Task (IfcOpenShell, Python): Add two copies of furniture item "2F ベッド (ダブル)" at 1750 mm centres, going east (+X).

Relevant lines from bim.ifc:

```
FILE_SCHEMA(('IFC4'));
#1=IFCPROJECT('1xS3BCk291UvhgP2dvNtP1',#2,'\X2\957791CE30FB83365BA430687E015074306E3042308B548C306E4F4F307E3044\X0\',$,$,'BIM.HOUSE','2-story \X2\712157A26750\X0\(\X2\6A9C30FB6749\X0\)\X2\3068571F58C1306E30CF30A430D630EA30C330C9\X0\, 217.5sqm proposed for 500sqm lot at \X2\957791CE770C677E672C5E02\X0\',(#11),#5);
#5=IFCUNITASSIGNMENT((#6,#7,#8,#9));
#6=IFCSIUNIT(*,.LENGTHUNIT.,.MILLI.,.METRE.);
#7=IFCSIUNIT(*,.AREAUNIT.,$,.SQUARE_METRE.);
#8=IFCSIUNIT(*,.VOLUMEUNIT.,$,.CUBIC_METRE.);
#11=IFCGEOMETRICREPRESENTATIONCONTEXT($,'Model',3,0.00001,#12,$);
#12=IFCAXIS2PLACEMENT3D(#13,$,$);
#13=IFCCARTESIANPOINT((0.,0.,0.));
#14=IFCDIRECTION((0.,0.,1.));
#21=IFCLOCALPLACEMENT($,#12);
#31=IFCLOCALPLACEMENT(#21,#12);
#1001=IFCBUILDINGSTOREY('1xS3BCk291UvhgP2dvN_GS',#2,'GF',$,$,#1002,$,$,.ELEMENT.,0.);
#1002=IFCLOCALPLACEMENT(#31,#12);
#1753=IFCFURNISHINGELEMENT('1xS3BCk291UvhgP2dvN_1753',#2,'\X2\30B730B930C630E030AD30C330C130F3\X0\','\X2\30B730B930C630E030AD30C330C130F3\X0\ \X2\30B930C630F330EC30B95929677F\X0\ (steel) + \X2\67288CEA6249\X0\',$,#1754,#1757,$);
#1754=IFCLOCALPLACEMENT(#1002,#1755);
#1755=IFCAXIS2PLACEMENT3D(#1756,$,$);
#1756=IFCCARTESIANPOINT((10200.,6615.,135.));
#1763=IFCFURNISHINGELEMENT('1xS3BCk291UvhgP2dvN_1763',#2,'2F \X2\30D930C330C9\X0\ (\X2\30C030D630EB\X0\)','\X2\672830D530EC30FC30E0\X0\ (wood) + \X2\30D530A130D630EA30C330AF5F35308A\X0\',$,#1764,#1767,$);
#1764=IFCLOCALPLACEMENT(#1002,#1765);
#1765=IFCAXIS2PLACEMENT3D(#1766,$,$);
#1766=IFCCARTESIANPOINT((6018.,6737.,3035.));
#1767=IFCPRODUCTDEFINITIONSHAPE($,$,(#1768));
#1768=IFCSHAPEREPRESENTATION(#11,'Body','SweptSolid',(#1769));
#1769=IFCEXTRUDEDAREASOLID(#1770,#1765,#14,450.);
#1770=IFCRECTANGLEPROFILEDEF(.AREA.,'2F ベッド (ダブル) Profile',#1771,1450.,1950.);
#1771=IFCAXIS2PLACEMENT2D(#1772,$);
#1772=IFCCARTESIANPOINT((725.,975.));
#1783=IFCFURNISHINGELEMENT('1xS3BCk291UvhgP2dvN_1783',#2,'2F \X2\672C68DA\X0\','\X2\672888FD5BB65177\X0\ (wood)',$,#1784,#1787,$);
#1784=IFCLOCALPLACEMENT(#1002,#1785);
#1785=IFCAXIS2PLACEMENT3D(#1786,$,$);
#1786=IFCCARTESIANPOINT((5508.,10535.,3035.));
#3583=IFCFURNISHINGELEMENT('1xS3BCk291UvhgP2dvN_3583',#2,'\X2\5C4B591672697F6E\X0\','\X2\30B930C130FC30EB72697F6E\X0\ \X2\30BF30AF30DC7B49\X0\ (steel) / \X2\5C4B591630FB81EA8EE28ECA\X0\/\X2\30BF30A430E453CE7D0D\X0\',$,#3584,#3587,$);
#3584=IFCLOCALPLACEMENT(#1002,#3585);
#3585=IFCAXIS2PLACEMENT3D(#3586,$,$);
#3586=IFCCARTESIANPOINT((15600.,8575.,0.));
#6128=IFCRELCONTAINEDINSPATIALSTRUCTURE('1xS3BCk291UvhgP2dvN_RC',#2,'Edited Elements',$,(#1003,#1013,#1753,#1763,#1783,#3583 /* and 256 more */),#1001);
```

```python
import numpy as np
import ifcopenshell
import ifcopenshell.api.geometry
import ifcopenshell.api.root
import ifcopenshell.util.element
import ifcopenshell.util.placement
import ifcopenshell.util.unit

model = ifcopenshell.open("bim.ifc")
unit_scale = ifcopenshell.util.unit.calculate_unit_scale(model)


def reuse_history(source, copy):
    """copy_class also copies each property set's owner history, people and application; keep the originals."""
    for rel in copy.IsDefinedBy:
        if rel.is_a("IfcRelDefinesByProperties") and (history := rel.RelatingPropertyDefinition.OwnerHistory):
            rel.RelatingPropertyDefinition.OwnerHistory = source.OwnerHistory
            ifcopenshell.util.element.remove_deep2(model, history)


source = model.by_guid("1xS3BCk291UvhgP2dvN_1763")
base = ifcopenshell.util.placement.get_local_placement(source.ObjectPlacement)
step = np.array([1.0, 0.0, 0.0]) * 1.75 / unit_scale

for i in range(1, 3):
    copy = ifcopenshell.api.root.copy_class(model, product=source)
    copy.Representation = ifcopenshell.util.element.copy_deep(
        model, source.Representation, exclude=["IfcGeometricRepresentationContext", "IfcRepresentationMap"]
    )
    reuse_history(source, copy)
    matrix = base.copy()
    matrix[:3, 3] += i * step
    print("added at", matrix[:3, 3].round(3) + 0.0)
    ifcopenshell.api.geometry.edit_object_placement(model, product=copy, matrix=matrix, is_si=False)

model.write("bim_edited.ifc")
```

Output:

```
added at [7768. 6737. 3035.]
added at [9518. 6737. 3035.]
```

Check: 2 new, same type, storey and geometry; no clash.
